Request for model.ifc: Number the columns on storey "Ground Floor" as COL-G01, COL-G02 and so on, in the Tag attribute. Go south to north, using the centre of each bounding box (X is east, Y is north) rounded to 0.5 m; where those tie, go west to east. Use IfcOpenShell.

First a look at what the model holds.

```python
import ifcopenshell
import ifcopenshell.util.element
import ifcopenshell.util.placement

model = ifcopenshell.open("model.ifc")
print(model.schema)
storey = next(s for s in model.by_type("IfcBuildingStorey") if s.Name == "Ground Floor")
columns = [e for e in ifcopenshell.util.element.get_decomposition(storey) if e.is_a("IfcColumn")]
for e in sorted(columns, key=lambda e: e.id()):
    origin = ifcopenshell.util.placement.get_local_placement(e.ObjectPlacement)[:3, 3]
    print(e.id(), e.Tag, e.Name, origin.round(2) + 0.0, sep=" | ")
```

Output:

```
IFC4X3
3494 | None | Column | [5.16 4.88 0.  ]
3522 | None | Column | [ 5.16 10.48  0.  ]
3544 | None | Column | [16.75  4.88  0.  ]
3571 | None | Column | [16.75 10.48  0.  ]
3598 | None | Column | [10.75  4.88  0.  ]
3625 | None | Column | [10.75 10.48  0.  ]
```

```python
import ifcopenshell
import ifcopenshell.geom
import ifcopenshell.util.element
import ifcopenshell.util.shape

model = ifcopenshell.open("model.ifc")
settings = ifcopenshell.geom.settings()
settings.set("use-world-coords", True)


def centre(element):
    shape = ifcopenshell.geom.create_shape(settings, element)
    return ifcopenshell.util.shape.get_bbox_centroid(shape.geometry)


storey = next(s for s in model.by_type("IfcBuildingStorey") if s.Name == "Ground Floor")
columns = [e for e in ifcopenshell.util.element.get_decomposition(storey) if e.is_a("IfcColumn")]

# Insertion points can sit at a corner or the storey origin, so sort by the geometry (in metres).
centres = {e: centre(e) for e in columns}
columns.sort(key=lambda e: (round(centres[e][1] / 0.5), centres[e][0]))

for i, e in enumerate(columns, start=1):
    number = f"COL-G{i:02d}"
    e.Tag = number
    print(e.id(), number)

model.write("model_rev.ifc")
```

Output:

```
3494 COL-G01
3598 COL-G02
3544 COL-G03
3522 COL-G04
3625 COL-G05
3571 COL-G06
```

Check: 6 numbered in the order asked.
